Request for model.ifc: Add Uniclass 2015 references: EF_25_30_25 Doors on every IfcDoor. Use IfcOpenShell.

First a look at what the model holds.

```python
import ifcopenshell

model = ifcopenshell.open("model.ifc")
print(model.schema)
print("classifications:", [c.Name for c in model.by_type("IfcClassification")])
for ifc_class in ("IfcDoor", "IfcRoof", "IfcStair", "IfcWall", "IfcWindow"):
    print(ifc_class, len(model.by_type(ifc_class)))
```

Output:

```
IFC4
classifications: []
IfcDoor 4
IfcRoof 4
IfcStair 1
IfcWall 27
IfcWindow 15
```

```python
import ifcopenshell
import ifcopenshell.api.classification

model = ifcopenshell.open("model.ifc")

system = ifcopenshell.api.classification.add_classification(model, classification="Uniclass 2015")

codes = {
    "IfcDoor": ("EF_25_30_25", "Doors"),
}
for ifc_class, (code, name) in codes.items():
    products = model.by_type(ifc_class)
    ifcopenshell.api.classification.add_reference(
        model, products=products, classification=system, identification=code, name=name
    )
    print(code, len(products))

model.write("model_rev.ifc")
```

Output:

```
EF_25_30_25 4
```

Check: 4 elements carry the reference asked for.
